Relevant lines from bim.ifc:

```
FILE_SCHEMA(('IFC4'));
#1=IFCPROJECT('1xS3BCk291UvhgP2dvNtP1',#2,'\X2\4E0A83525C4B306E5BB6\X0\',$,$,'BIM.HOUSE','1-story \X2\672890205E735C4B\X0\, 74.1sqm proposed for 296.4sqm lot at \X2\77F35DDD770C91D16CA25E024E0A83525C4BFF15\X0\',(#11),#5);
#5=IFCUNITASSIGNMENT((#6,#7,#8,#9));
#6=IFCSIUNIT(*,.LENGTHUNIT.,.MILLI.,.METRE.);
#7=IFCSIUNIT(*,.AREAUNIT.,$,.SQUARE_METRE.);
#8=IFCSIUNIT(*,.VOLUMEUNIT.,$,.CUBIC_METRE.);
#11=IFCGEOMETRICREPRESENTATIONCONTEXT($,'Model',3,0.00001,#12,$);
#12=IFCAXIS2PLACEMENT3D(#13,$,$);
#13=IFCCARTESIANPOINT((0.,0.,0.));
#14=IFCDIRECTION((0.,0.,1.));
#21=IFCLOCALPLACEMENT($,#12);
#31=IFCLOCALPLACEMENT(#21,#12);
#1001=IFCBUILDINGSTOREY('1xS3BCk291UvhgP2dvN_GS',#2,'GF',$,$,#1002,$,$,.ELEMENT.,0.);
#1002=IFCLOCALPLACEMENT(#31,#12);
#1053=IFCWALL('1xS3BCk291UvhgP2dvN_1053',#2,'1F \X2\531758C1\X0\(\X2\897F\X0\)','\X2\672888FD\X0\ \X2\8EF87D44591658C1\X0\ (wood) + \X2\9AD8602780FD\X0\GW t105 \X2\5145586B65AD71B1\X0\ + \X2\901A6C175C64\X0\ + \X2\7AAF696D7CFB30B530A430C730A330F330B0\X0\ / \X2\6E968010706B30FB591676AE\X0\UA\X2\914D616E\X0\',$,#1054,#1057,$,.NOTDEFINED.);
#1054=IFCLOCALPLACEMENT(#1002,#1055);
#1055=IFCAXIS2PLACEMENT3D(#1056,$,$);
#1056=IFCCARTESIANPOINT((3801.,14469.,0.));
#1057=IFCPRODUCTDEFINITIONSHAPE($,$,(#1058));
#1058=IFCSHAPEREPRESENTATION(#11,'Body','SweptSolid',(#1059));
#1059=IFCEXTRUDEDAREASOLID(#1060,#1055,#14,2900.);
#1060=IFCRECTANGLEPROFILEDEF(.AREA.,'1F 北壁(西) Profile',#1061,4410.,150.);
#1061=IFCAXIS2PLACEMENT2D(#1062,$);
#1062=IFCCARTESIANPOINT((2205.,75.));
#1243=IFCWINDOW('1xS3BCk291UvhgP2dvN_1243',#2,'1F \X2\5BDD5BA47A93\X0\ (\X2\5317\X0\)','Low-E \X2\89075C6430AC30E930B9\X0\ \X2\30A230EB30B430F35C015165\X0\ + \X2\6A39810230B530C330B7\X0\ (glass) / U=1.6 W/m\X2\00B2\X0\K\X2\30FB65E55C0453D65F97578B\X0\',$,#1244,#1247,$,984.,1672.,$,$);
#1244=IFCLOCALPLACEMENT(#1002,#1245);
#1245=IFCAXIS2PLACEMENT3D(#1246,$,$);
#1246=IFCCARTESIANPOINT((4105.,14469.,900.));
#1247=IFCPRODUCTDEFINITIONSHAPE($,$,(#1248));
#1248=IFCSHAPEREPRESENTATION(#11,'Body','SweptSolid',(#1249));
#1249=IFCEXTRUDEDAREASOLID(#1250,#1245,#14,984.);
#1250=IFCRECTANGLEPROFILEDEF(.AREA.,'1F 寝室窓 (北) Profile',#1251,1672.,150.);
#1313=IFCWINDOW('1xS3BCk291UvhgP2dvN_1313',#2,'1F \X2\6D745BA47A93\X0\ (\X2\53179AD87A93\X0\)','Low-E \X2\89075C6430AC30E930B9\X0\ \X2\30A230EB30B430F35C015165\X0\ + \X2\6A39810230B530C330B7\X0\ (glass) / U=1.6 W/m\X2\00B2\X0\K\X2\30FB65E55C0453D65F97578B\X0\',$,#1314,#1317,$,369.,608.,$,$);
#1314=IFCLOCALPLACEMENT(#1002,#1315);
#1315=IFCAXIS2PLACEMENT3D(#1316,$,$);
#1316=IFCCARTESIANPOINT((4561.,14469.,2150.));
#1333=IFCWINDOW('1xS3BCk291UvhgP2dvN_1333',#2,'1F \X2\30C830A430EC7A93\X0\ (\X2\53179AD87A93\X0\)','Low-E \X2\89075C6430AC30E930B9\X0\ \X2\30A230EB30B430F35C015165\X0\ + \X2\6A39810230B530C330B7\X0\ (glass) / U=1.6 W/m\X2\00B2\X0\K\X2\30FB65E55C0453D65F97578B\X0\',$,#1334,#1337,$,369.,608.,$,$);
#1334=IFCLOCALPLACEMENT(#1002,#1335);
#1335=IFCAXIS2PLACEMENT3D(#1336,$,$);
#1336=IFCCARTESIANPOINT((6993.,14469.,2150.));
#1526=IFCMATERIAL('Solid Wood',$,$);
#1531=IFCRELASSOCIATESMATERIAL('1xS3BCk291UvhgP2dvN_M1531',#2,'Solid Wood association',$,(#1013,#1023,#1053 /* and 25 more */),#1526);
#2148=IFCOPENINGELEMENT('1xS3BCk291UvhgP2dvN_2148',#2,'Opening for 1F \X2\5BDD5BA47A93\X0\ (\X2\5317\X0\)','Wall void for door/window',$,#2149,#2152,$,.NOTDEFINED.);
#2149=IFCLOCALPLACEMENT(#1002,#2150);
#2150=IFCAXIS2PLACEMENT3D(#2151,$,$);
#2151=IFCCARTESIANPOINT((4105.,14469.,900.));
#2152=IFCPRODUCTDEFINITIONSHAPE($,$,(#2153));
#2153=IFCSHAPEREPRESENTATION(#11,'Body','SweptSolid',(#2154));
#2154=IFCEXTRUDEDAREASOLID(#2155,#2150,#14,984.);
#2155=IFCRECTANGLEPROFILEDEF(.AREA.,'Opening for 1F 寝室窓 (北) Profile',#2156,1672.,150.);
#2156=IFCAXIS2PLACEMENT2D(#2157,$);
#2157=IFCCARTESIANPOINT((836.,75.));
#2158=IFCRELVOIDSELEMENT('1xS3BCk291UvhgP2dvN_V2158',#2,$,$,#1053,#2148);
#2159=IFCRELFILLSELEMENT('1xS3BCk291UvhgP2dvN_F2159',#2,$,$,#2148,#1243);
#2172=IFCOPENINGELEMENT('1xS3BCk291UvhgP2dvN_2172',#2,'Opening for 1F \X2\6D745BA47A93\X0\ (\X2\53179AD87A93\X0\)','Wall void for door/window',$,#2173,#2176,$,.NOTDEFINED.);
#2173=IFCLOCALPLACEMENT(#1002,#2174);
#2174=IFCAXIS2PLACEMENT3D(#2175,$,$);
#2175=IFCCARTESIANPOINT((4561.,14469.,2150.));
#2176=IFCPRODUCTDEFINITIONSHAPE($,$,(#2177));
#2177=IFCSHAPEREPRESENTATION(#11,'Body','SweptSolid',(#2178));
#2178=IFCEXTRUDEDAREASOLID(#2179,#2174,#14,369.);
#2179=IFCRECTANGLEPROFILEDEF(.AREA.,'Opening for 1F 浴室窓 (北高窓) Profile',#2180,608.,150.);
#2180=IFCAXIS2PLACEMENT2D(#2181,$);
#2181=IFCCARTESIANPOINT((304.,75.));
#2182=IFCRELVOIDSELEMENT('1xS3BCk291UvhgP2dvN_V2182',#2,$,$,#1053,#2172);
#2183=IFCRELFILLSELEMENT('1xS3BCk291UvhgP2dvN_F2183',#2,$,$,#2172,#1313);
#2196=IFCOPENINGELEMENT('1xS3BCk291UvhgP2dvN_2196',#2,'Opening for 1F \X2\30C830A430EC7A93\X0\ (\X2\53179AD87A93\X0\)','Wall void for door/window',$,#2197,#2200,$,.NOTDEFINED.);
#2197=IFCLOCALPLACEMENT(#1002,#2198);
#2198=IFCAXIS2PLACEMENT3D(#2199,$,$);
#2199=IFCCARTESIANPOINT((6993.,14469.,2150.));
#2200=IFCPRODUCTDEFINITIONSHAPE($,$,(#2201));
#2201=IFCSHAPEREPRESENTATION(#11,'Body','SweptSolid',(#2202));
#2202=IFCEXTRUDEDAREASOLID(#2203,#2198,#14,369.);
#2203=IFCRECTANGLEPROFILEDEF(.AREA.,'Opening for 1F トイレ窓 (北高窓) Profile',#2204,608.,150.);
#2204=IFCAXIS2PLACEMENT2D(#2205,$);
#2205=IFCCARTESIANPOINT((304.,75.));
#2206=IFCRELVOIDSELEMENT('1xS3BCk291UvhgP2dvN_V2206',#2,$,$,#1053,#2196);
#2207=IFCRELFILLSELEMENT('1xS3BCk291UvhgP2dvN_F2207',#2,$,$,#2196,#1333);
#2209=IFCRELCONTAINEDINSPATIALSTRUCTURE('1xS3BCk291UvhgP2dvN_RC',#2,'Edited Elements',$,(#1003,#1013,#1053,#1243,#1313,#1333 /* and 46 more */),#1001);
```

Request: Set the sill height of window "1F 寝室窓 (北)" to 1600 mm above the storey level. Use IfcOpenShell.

```python
import numpy as np
import ifcopenshell
import ifcopenshell.api.geometry
import ifcopenshell.geom
import ifcopenshell.util.element
import ifcopenshell.util.placement
import ifcopenshell.util.shape
import ifcopenshell.util.unit

model = ifcopenshell.open("bim.ifc")
unit_scale = ifcopenshell.util.unit.calculate_unit_scale(model)

window = model.by_guid("1xS3BCk291UvhgP2dvN_1243")
opening = window.FillsVoids[0].RelatingOpeningElement
storey = ifcopenshell.util.element.get_container(window, ifc_class="IfcBuildingStorey")
level = ifcopenshell.util.placement.get_local_placement(storey.ObjectPlacement)[2, 3]

# The opening's origin need not be at the sill, so measure its lowest point.
shape = ifcopenshell.geom.create_shape(ifcopenshell.geom.settings(), opening)
bottom = ifcopenshell.util.shape.get_shape_bottom_elevation(shape, shape.geometry) / unit_scale
dz = level + 1600.0 - bottom

shift = np.array([0.0, 0.0, dz])
# The window is not placed relative to its opening, so move both.
for product in (opening, window):
    matrix = ifcopenshell.util.placement.get_local_placement(product.ObjectPlacement)
    matrix[:3, 3] += shift
    ifcopenshell.api.geometry.edit_object_placement(model, product=product, matrix=matrix, is_si=False)

print(f"moved by {dz * unit_scale:+.3f} m")

model.write("bim_updated.ifc")
```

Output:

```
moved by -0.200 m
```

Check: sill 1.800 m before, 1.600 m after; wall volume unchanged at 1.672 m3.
